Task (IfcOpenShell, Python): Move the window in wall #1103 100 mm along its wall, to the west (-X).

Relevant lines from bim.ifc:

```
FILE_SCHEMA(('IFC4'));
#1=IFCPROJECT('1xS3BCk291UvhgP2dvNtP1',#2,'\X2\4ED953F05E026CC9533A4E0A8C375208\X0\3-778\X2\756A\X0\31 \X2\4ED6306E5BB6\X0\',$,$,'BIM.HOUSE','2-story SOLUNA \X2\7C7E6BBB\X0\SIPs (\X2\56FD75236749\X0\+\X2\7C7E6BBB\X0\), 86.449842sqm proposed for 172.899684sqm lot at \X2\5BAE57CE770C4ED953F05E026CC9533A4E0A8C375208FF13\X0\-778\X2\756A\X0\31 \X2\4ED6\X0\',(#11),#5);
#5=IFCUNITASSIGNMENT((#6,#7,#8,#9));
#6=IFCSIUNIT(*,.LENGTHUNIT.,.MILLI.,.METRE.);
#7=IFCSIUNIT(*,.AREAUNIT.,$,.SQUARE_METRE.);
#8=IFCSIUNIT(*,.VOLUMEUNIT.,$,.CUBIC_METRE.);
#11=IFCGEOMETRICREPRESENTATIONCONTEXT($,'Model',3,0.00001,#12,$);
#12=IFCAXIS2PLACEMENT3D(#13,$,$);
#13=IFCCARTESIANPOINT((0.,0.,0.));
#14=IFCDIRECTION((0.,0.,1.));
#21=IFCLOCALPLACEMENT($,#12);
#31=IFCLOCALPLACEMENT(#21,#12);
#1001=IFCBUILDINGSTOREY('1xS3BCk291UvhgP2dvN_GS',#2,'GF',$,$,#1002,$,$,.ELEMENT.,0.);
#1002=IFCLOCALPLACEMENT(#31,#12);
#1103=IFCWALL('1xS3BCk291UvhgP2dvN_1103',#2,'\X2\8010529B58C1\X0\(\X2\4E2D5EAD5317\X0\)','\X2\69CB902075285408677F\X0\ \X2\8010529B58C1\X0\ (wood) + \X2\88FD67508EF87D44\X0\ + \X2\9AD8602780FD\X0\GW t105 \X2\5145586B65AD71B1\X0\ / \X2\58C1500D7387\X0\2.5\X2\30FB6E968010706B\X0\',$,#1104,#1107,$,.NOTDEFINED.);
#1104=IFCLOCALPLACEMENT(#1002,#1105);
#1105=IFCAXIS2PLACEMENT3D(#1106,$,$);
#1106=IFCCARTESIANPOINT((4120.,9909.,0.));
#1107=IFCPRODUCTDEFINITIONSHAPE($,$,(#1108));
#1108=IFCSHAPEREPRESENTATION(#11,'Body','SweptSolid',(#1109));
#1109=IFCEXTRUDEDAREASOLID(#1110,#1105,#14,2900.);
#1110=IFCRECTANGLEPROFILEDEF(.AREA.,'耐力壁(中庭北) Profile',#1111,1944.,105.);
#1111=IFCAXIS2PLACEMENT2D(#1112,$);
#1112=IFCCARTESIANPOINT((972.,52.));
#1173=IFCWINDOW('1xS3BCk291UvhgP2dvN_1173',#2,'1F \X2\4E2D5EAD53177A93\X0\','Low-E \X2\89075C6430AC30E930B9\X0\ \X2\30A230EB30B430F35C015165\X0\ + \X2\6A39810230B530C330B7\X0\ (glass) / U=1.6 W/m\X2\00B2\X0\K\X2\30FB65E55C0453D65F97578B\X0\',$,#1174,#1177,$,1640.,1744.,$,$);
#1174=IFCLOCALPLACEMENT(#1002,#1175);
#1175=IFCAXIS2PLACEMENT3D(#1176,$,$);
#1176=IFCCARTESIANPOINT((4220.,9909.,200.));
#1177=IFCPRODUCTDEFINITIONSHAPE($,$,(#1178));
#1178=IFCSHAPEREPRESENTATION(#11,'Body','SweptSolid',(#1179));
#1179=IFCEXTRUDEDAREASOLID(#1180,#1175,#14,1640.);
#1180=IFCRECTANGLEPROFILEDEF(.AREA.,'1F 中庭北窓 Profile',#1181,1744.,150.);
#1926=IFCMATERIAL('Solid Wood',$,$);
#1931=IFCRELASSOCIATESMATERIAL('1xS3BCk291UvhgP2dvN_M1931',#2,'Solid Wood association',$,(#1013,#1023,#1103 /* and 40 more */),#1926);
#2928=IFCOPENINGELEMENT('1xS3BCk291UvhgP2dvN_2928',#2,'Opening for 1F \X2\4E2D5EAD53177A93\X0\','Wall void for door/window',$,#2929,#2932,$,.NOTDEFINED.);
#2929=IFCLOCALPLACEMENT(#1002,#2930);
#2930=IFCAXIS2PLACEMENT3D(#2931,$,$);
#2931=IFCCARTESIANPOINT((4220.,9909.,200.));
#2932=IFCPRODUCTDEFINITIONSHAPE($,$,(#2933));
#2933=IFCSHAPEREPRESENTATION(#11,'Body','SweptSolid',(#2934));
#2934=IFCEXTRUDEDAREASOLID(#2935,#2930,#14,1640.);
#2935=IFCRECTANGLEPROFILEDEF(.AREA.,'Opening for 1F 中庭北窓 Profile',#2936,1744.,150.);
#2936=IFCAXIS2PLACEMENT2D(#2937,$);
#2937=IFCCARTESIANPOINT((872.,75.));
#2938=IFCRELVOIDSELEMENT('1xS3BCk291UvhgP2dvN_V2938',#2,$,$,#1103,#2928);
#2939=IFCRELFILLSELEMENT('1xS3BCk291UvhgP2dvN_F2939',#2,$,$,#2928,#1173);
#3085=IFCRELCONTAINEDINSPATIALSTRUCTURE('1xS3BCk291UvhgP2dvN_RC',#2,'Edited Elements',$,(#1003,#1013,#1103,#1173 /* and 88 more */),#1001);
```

```python
import ifcopenshell
import ifcopenshell.api.geometry
import ifcopenshell.util.placement
import ifcopenshell.util.unit

model = ifcopenshell.open("bim.ifc")
unit_scale = ifcopenshell.util.unit.calculate_unit_scale(model)

window = model.by_guid("1xS3BCk291UvhgP2dvN_1173")
opening = window.FillsVoids[0].RelatingOpeningElement
wall = opening.VoidsElements[0].RelatingBuildingElement

wall_matrix = ifcopenshell.util.placement.get_local_placement(wall.ObjectPlacement)
shift = wall_matrix[:3, 0] * -0.1 / unit_scale
before = ifcopenshell.util.placement.get_local_placement(window.ObjectPlacement)[:3, 3].copy()

# The window is not placed relative to its opening, so move both.
for product in (opening, window):
    matrix = ifcopenshell.util.placement.get_local_placement(product.ObjectPlacement)
    matrix[:3, 3] += shift
    ifcopenshell.api.geometry.edit_object_placement(model, product=product, matrix=matrix, is_si=False)

after = ifcopenshell.util.placement.get_local_placement(window.ObjectPlacement)[:3, 3]
print("window moved by", (after - before).round(3) + 0.0)

model.write("bim-out.ifc")
```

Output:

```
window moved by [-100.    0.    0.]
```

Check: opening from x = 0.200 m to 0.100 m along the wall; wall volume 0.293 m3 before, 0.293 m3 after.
